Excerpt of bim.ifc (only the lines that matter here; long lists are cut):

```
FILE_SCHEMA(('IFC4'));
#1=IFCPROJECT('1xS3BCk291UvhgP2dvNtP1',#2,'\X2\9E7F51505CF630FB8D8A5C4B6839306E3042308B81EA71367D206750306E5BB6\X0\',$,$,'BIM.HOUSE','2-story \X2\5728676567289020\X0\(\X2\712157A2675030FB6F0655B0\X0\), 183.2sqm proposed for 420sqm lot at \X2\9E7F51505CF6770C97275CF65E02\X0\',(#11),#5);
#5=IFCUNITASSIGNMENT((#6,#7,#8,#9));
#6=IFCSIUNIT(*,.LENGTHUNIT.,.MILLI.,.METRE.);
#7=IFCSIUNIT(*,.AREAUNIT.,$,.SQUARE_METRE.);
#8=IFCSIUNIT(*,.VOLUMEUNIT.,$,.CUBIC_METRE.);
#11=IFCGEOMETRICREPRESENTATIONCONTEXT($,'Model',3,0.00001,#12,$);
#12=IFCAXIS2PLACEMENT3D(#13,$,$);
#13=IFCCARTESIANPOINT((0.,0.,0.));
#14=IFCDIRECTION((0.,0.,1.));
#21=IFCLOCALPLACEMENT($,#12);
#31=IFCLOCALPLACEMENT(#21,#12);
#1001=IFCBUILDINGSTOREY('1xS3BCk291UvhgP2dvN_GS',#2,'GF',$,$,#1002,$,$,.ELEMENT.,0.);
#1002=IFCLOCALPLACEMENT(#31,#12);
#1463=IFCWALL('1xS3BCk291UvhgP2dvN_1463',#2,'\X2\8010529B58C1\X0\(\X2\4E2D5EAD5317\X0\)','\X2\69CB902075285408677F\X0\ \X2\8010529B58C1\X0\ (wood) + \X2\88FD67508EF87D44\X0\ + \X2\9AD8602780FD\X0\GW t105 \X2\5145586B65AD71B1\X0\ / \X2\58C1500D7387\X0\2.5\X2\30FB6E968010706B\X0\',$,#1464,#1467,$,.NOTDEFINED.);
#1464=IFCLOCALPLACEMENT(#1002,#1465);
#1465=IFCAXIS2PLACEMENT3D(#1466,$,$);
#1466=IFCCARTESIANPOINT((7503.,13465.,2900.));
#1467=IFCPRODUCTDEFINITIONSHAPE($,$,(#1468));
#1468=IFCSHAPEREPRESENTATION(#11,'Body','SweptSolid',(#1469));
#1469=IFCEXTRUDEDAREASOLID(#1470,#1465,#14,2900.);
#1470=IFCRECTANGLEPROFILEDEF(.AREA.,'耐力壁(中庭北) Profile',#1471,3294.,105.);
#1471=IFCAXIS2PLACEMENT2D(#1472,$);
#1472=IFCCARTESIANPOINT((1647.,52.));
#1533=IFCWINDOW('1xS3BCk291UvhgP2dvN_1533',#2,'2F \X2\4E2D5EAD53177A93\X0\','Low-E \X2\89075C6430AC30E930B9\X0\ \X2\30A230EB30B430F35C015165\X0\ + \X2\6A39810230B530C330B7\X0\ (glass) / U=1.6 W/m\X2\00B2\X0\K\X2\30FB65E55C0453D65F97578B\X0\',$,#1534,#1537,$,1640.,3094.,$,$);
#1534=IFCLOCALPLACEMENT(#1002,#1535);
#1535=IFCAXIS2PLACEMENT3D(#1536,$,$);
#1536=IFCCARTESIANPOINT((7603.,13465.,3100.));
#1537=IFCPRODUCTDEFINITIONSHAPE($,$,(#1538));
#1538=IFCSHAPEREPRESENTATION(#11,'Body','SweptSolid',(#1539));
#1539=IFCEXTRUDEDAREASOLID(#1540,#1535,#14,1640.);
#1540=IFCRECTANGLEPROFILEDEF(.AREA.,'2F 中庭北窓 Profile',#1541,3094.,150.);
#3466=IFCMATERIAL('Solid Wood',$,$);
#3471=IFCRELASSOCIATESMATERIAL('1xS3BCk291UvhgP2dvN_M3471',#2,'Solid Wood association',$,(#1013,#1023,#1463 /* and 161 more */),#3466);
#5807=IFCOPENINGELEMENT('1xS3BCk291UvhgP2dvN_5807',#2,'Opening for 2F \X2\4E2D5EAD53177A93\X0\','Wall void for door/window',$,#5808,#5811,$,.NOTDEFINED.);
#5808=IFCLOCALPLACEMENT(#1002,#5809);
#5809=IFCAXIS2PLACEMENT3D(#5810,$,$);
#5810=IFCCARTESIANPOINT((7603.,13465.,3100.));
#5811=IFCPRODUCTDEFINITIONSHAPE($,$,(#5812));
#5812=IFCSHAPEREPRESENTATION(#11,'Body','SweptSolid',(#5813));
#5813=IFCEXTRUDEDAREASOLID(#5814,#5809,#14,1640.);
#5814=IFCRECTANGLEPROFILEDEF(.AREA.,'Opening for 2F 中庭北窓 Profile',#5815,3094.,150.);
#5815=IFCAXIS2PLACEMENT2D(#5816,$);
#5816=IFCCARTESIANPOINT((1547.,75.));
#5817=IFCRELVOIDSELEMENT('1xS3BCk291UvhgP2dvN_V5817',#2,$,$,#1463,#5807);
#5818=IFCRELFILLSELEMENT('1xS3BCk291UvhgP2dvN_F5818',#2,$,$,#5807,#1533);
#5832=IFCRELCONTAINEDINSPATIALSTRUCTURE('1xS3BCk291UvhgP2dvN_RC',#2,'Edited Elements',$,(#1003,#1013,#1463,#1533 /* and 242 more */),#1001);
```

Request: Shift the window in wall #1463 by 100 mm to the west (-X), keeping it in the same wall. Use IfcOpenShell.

```python
import ifcopenshell
import ifcopenshell.api.geometry
import ifcopenshell.util.placement

model = ifcopenshell.open("bim.ifc")

window = model.by_guid("1xS3BCk291UvhgP2dvN_1533")
opening = window.FillsVoids[0].RelatingOpeningElement
wall = opening.VoidsElements[0].RelatingBuildingElement

wall_matrix = ifcopenshell.util.placement.get_local_placement(wall.ObjectPlacement)
shift = wall_matrix[:3, 0] * -100.0
before = ifcopenshell.util.placement.get_local_placement(window.ObjectPlacement)[:3, 3].copy()

# The window is not placed relative to its opening, so move both.
for product in (opening, window):
    matrix = ifcopenshell.util.placement.get_local_placement(product.ObjectPlacement)
    matrix[:3, 3] += shift
    ifcopenshell.api.geometry.edit_object_placement(model, product=product, matrix=matrix, is_si=False)

after = ifcopenshell.util.placement.get_local_placement(window.ObjectPlacement)[:3, 3]
print("window moved by", (after - before).round(3) + 0.0)

model.write("bim_updated.ifc")
```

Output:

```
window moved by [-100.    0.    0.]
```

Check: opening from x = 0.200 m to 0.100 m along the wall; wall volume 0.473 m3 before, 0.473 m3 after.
